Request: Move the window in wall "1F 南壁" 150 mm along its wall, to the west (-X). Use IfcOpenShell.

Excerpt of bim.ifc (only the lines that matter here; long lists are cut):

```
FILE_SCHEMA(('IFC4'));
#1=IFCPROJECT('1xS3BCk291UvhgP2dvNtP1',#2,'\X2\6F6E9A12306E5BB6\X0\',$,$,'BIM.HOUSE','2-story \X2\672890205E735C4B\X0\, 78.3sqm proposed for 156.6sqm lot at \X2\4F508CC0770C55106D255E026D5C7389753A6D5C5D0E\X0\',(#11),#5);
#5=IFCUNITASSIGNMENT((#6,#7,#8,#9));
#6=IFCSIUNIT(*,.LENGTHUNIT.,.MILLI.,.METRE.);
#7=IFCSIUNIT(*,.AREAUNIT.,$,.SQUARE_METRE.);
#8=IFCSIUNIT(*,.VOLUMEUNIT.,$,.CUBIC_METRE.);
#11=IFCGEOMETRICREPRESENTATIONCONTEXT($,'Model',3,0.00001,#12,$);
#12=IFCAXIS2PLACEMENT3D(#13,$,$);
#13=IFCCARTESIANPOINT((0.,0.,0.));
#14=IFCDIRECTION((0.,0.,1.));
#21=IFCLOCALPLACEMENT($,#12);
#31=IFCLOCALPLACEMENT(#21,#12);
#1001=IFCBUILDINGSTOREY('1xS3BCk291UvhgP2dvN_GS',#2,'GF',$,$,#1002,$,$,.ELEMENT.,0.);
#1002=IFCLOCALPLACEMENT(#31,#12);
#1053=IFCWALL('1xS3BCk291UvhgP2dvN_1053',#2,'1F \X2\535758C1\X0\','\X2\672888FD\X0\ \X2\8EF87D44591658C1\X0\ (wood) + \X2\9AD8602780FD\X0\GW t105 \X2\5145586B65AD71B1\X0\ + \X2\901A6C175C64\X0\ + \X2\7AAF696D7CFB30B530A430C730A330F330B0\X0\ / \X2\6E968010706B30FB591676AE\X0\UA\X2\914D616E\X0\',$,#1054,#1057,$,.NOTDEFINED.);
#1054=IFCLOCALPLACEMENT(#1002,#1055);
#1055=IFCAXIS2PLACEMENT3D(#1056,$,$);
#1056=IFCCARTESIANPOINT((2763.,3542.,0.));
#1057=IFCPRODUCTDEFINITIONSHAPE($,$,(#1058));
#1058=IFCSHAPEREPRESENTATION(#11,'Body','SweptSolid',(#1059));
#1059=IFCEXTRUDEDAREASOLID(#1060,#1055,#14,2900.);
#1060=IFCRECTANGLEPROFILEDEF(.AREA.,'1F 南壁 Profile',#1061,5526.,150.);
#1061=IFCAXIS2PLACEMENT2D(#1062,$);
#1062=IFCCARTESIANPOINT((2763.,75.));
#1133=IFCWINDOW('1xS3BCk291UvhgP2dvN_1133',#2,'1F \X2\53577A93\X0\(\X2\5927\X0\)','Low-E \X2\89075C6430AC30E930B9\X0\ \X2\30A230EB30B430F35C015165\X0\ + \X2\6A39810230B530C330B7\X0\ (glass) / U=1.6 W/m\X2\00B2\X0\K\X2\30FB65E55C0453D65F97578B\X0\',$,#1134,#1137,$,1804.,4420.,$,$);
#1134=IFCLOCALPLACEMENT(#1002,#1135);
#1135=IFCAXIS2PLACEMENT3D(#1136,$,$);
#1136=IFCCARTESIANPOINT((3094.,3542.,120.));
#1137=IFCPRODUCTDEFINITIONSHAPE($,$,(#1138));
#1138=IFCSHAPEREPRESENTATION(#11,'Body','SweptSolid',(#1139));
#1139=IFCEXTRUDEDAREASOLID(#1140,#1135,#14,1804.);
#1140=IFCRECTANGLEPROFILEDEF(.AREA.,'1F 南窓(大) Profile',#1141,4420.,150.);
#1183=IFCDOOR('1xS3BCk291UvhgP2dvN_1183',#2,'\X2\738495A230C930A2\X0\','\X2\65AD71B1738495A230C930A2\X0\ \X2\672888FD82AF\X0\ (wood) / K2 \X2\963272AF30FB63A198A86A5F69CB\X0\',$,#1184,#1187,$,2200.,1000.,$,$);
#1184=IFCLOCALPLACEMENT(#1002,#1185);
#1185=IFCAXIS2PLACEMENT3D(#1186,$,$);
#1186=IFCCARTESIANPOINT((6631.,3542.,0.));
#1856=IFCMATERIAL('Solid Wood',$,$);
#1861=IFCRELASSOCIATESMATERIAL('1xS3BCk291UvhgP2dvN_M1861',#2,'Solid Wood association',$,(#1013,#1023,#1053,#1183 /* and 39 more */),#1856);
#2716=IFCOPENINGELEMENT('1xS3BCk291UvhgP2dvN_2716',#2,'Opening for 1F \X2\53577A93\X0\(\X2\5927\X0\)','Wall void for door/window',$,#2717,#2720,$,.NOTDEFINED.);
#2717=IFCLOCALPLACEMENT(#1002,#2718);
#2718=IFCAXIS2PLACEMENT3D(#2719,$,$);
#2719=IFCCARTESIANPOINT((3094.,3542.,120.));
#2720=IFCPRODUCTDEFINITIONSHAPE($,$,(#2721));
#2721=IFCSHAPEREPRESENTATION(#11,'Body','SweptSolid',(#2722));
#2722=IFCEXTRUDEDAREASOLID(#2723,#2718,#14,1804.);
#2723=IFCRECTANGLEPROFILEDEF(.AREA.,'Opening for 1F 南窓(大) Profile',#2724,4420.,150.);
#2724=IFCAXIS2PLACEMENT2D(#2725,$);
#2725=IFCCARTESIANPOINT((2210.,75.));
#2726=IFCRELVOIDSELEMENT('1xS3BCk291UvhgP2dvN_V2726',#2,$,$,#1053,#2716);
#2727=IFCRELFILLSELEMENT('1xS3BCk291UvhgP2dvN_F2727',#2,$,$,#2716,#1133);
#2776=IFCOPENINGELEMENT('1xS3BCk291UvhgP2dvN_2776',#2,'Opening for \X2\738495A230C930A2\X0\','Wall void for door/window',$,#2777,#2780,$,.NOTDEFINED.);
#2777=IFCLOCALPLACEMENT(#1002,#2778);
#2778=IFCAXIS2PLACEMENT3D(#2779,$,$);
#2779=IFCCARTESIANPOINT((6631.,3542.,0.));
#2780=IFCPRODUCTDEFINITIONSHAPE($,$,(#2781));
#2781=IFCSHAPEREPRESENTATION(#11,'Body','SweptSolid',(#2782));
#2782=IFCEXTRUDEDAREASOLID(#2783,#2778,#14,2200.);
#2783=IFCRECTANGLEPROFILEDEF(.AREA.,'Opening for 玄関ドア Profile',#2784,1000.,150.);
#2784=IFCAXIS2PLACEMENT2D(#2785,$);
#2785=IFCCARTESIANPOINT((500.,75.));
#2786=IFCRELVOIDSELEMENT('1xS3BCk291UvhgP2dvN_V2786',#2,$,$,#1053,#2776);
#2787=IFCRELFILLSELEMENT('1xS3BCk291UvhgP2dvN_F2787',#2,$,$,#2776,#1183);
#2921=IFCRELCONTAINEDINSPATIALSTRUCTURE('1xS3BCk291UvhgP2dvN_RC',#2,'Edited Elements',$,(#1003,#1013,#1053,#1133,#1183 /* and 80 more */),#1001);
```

```python
import ifcopenshell
import ifcopenshell.api.geometry
import ifcopenshell.util.placement
import ifcopenshell.util.unit

model = ifcopenshell.open("bim.ifc")
unit_scale = ifcopenshell.util.unit.calculate_unit_scale(model)

window = model.by_guid("1xS3BCk291UvhgP2dvN_1133")
opening = window.FillsVoids[0].RelatingOpeningElement
wall = opening.VoidsElements[0].RelatingBuildingElement

wall_matrix = ifcopenshell.util.placement.get_local_placement(wall.ObjectPlacement)
shift = wall_matrix[:3, 0] * -0.15 / unit_scale
before = ifcopenshell.util.placement.get_local_placement(window.ObjectPlacement)[:3, 3].copy()

# The window is not placed relative to its opening, so move both.
for product in (opening, window):
    matrix = ifcopenshell.util.placement.get_local_placement(product.ObjectPlacement)
    matrix[:3, 3] += shift
    ifcopenshell.api.geometry.edit_object_placement(model, product=product, matrix=matrix, is_si=False)

after = ifcopenshell.util.placement.get_local_placement(window.ObjectPlacement)[:3, 3]
print("window moved by", (after - before).round(3) + 0.0)

model.write("bim_updated.ifc")
```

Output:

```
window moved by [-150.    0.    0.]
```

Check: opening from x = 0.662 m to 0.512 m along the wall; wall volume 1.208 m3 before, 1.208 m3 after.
